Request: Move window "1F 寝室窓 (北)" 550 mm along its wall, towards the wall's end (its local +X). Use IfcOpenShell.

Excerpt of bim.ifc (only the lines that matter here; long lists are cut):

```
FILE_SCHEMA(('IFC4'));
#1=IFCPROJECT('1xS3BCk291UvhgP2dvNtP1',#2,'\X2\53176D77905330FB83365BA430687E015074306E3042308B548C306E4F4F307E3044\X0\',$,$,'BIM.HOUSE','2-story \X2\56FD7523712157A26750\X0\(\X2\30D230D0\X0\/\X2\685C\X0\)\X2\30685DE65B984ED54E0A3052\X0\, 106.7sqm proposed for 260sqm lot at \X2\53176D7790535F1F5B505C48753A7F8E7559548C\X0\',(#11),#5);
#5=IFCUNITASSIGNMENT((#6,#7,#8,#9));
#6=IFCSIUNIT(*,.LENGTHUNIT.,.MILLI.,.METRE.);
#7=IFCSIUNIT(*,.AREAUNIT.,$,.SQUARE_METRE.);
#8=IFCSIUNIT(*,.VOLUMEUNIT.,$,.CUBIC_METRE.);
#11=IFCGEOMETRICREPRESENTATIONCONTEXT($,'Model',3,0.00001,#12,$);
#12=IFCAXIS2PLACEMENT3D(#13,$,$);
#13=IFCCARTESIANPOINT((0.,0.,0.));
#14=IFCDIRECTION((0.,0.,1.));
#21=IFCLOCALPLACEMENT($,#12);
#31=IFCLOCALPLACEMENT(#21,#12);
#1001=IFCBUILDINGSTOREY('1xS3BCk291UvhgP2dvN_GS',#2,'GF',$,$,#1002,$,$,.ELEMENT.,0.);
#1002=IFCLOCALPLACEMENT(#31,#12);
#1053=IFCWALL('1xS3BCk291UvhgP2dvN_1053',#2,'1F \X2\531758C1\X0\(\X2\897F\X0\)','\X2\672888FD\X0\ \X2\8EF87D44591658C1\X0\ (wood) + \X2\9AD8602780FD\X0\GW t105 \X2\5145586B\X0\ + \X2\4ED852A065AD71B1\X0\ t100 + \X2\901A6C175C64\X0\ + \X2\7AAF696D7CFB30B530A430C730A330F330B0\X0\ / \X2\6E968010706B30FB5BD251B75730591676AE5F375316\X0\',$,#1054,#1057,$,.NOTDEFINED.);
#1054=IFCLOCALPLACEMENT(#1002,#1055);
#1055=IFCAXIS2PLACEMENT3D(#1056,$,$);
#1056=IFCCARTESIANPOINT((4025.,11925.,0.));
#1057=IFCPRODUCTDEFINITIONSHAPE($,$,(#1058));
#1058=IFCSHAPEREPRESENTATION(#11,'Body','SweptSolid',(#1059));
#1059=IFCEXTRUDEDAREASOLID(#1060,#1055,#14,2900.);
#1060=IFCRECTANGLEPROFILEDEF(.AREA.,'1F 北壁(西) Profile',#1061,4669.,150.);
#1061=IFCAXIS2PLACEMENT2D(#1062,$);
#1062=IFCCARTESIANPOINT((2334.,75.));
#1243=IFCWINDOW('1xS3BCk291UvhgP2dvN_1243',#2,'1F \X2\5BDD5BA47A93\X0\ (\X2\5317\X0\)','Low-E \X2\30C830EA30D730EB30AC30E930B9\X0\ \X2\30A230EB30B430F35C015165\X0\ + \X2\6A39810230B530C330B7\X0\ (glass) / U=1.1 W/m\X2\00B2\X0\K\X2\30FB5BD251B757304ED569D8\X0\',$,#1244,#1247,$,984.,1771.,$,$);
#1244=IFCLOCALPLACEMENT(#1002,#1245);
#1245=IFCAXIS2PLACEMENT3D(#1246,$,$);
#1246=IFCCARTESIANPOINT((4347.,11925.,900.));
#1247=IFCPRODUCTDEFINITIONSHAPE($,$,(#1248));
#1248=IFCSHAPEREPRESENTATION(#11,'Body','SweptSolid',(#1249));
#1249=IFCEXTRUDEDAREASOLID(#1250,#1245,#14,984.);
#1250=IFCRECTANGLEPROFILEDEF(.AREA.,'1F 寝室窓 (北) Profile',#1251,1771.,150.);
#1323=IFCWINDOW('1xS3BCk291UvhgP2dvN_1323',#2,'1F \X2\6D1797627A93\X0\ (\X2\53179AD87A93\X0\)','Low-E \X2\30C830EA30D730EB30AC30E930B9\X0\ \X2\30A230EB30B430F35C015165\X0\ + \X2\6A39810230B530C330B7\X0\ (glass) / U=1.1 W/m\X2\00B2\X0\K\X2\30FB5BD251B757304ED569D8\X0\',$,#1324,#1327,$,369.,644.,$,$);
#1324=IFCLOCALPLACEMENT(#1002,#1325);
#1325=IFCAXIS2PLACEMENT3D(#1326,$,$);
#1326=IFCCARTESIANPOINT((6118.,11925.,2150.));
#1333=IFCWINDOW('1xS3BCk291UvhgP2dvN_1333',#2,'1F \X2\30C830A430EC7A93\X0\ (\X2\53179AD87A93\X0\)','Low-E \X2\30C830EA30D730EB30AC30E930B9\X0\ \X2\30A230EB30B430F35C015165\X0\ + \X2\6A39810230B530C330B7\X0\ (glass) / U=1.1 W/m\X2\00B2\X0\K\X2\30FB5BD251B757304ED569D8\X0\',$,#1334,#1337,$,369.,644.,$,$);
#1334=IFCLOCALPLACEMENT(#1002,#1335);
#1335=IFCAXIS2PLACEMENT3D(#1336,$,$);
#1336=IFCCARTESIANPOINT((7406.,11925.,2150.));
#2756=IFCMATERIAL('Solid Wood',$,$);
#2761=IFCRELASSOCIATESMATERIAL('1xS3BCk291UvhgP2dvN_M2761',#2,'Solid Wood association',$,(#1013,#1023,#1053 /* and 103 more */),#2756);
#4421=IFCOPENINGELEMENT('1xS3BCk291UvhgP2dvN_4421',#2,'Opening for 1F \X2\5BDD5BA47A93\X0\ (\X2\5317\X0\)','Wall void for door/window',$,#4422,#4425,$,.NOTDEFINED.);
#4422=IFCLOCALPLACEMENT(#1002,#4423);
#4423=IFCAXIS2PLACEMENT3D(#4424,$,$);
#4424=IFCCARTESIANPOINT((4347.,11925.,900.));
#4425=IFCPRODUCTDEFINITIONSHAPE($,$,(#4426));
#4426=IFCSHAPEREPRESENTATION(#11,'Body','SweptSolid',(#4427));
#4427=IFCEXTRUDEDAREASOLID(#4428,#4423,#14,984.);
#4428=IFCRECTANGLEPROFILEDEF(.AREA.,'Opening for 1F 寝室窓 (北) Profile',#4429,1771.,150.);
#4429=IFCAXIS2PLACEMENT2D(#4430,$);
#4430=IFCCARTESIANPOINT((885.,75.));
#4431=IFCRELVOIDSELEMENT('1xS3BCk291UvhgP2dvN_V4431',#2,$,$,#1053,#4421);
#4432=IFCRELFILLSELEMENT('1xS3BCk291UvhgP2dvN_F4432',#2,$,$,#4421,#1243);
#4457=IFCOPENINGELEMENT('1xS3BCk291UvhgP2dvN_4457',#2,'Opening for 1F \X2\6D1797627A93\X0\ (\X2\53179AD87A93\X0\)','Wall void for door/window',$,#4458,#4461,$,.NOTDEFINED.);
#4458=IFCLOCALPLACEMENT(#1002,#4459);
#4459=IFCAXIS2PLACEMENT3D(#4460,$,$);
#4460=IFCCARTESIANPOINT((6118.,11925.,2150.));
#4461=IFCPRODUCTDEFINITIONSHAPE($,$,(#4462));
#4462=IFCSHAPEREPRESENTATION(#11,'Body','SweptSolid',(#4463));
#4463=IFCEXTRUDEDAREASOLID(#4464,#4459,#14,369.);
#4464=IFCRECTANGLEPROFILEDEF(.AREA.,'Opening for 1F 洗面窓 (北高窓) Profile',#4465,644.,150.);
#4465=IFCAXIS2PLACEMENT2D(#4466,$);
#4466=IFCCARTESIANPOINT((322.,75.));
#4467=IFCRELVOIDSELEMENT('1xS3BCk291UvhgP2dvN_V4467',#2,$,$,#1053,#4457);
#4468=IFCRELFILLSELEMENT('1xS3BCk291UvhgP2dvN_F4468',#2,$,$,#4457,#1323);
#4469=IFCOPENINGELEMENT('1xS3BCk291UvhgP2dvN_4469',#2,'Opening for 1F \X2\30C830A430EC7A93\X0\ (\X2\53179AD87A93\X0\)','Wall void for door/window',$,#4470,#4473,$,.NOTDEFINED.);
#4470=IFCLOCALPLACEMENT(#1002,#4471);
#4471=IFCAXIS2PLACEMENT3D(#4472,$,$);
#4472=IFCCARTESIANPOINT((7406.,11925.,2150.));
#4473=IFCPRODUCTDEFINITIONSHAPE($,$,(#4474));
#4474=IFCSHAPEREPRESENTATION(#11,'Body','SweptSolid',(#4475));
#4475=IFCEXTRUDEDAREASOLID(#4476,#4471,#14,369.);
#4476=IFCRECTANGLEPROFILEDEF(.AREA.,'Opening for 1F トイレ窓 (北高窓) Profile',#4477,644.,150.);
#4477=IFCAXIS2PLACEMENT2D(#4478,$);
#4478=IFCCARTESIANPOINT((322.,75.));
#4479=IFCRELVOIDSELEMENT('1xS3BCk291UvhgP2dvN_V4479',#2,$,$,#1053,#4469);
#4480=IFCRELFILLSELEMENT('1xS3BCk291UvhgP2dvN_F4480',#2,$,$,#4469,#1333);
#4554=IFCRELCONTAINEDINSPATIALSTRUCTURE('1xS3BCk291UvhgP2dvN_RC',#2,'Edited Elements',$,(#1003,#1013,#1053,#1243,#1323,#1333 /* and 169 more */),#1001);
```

```python
import ifcopenshell
import ifcopenshell.api.geometry
import ifcopenshell.util.placement

model = ifcopenshell.open("bim.ifc")

window = model.by_guid("1xS3BCk291UvhgP2dvN_1243")
opening = window.FillsVoids[0].RelatingOpeningElement
wall = opening.VoidsElements[0].RelatingBuildingElement

wall_matrix = ifcopenshell.util.placement.get_local_placement(wall.ObjectPlacement)
shift = wall_matrix[:3, 0] * 550.0
before = ifcopenshell.util.placement.get_local_placement(window.ObjectPlacement)[:3, 3].copy()

# The window is not placed relative to its opening, so move both.
for product in (opening, window):
    matrix = ifcopenshell.util.placement.get_local_placement(product.ObjectPlacement)
    matrix[:3, 3] += shift
    ifcopenshell.api.geometry.edit_object_placement(model, product=product, matrix=matrix, is_si=False)

after = ifcopenshell.util.placement.get_local_placement(window.ObjectPlacement)[:3, 3]
print("window moved by", (after - before).round(3) + 0.0)

model.write("bim_rev.ifc")
```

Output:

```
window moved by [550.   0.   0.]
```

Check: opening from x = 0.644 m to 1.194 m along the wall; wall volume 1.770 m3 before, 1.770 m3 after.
